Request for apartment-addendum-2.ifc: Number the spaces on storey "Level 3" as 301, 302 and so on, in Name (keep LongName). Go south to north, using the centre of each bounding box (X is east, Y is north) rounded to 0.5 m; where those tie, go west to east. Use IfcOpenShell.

First a look at what the model holds.

```python
import ifcopenshell
import ifcopenshell.util.element
import ifcopenshell.util.placement

model = ifcopenshell.open("apartment-addendum-2.ifc")
print(model.schema)
storey = next(s for s in model.by_type("IfcBuildingStorey") if s.Name == "Level 3")
spaces = [e for e in ifcopenshell.util.element.get_decomposition(storey) if e.is_a("IfcSpace")]
for e in sorted(spaces, key=lambda e: e.id()):
    origin = ifcopenshell.util.placement.get_local_placement(e.ObjectPlacement)[:3, 3]
    print(e.id(), e.Name, e.LongName, origin.round(2) + 0.0, sep=" | ")
```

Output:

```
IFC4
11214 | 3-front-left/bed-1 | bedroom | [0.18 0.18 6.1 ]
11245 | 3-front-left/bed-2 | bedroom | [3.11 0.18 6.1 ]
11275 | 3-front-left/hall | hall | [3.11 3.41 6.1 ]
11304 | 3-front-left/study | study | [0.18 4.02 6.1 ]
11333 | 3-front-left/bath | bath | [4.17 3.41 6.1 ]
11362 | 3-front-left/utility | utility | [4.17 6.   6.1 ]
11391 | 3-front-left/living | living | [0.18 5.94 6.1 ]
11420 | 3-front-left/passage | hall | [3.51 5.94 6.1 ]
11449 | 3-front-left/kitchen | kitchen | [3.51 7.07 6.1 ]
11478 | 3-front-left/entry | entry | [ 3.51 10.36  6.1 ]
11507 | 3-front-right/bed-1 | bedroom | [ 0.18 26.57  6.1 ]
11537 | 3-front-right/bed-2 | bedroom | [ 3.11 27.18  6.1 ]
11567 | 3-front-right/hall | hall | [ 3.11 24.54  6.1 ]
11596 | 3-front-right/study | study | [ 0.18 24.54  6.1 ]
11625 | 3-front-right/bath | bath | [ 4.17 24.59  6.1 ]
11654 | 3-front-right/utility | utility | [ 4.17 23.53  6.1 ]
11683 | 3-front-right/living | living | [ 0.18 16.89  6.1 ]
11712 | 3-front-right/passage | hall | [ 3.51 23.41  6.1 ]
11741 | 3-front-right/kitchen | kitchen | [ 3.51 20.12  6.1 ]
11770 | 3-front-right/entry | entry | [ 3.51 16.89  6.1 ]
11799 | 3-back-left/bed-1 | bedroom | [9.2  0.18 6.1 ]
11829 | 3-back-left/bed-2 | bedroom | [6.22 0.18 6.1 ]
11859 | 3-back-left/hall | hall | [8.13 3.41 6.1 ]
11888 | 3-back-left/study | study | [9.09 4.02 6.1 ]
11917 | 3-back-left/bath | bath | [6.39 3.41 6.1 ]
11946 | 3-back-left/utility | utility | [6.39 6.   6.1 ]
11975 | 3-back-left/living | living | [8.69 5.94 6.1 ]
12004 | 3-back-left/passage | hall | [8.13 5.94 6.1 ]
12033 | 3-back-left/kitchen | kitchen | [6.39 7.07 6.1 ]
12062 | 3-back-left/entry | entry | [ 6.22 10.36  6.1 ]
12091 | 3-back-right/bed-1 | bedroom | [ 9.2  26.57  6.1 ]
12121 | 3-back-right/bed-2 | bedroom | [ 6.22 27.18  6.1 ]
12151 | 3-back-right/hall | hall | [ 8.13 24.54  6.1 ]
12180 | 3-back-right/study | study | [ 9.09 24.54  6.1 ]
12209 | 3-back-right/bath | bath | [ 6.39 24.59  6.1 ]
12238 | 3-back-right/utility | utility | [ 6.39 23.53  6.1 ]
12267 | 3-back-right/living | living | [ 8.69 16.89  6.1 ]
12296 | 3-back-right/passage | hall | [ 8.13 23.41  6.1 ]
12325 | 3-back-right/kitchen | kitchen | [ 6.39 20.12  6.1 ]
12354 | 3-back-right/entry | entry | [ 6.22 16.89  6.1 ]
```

```python
import ifcopenshell
import ifcopenshell.geom
import ifcopenshell.util.element
import ifcopenshell.util.shape

model = ifcopenshell.open("apartment-addendum-2.ifc")
settings = ifcopenshell.geom.settings()
settings.set("use-world-coords", True)


def centre(element):
    shape = ifcopenshell.geom.create_shape(settings, element)
    return ifcopenshell.util.shape.get_bbox_centroid(shape.geometry)


storey = next(s for s in model.by_type("IfcBuildingStorey") if s.Name == "Level 3")
spaces = [e for e in ifcopenshell.util.element.get_decomposition(storey) if e.is_a("IfcSpace")]

# Insertion points can sit at a corner or the storey origin, so sort by the geometry (in metres).
centres = {e: centre(e) for e in spaces}
spaces.sort(key=lambda e: (round(centres[e][1] / 0.5), centres[e][0]))

for i, e in enumerate(spaces, start=1):
    number = f"3{i:02d}"
    e.Name = number
    print(e.id(), number)

model.write("apartment-addendum-2-out.ifc")
```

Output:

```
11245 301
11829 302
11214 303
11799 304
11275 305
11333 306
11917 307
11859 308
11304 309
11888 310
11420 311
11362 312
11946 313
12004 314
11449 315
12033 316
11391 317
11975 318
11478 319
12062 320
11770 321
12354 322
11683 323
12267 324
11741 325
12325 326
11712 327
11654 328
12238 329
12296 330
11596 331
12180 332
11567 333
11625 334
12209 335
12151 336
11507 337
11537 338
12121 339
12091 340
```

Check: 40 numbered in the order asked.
